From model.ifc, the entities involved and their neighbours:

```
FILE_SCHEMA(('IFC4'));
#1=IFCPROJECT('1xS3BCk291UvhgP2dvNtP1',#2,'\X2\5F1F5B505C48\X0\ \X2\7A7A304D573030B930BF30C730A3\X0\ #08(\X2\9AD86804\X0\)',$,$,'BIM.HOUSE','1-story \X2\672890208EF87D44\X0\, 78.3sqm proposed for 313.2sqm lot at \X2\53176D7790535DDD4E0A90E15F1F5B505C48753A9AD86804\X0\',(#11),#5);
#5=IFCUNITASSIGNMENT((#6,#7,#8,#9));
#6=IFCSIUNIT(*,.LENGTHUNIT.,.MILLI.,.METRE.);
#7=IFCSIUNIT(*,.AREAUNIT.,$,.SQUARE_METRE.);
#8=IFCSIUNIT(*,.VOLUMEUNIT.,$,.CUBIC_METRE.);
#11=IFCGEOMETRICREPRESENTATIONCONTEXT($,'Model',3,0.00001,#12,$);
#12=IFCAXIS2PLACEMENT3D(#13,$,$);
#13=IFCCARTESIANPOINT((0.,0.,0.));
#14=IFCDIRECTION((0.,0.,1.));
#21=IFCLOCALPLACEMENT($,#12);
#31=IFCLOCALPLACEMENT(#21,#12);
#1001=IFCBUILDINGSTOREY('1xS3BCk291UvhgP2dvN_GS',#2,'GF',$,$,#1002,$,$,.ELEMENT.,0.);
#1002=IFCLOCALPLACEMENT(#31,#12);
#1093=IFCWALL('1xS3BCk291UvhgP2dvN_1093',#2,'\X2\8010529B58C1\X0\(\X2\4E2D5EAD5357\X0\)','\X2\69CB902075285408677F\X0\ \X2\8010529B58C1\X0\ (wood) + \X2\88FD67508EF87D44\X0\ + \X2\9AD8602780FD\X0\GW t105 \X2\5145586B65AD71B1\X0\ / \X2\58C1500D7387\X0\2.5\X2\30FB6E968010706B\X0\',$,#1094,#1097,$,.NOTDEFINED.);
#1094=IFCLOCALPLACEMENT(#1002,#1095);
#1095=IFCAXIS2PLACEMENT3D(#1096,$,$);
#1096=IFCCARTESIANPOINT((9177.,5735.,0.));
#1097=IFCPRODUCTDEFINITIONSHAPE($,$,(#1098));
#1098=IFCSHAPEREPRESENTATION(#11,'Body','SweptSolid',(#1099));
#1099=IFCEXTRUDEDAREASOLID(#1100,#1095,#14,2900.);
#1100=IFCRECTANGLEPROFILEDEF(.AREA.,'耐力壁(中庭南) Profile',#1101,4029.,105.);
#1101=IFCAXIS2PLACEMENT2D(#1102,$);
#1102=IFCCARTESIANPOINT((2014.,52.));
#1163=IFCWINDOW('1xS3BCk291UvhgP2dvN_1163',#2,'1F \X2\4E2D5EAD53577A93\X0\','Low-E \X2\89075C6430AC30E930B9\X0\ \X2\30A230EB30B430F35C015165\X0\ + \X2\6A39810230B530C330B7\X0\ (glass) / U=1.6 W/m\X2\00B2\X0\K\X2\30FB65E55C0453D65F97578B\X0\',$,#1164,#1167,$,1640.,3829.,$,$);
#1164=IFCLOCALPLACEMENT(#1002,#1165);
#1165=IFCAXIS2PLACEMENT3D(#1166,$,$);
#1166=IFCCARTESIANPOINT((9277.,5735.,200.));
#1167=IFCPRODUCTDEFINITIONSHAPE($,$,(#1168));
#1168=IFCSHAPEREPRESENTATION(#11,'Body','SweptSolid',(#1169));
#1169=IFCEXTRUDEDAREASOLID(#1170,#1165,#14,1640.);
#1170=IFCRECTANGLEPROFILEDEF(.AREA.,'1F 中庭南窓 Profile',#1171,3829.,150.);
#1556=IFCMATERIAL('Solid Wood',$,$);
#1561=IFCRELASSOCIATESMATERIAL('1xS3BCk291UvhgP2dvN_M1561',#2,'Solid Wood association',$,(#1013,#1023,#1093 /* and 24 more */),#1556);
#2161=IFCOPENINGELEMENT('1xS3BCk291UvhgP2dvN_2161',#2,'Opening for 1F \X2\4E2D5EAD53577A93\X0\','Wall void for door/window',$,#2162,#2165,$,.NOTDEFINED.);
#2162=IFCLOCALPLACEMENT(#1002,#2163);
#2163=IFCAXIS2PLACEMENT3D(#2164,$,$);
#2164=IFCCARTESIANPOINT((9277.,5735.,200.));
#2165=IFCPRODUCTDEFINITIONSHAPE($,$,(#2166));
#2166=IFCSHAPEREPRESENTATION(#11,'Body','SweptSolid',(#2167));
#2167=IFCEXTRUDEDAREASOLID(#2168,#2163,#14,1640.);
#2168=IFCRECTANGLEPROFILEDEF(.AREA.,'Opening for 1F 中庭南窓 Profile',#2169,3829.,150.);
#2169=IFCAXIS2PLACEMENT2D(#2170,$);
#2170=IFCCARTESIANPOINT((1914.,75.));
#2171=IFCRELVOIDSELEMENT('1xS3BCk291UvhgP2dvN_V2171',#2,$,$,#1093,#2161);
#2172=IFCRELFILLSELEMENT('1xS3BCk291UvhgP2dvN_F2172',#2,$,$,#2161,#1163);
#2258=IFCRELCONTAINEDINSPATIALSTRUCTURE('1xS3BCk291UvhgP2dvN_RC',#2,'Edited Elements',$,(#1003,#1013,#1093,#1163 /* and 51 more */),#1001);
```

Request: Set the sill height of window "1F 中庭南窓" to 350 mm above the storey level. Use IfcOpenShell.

```python
import numpy as np
import ifcopenshell
import ifcopenshell.api.geometry
import ifcopenshell.geom
import ifcopenshell.util.element
import ifcopenshell.util.placement
import ifcopenshell.util.shape
import ifcopenshell.util.unit

model = ifcopenshell.open("model.ifc")
unit_scale = ifcopenshell.util.unit.calculate_unit_scale(model)

window = model.by_guid("1xS3BCk291UvhgP2dvN_1163")
opening = window.FillsVoids[0].RelatingOpeningElement
storey = ifcopenshell.util.element.get_container(window, ifc_class="IfcBuildingStorey")
level = ifcopenshell.util.placement.get_local_placement(storey.ObjectPlacement)[2, 3]

# The opening's origin need not be at the sill, so measure its lowest point.
shape = ifcopenshell.geom.create_shape(ifcopenshell.geom.settings(), opening)
bottom = ifcopenshell.util.shape.get_shape_bottom_elevation(shape, shape.geometry) / unit_scale
dz = level + 350.0 - bottom

shift = np.array([0.0, 0.0, dz])
# The window is not placed relative to its opening, so move both.
for product in (opening, window):
    matrix = ifcopenshell.util.placement.get_local_placement(product.ObjectPlacement)
    matrix[:3, 3] += shift
    ifcopenshell.api.geometry.edit_object_placement(model, product=product, matrix=matrix, is_si=False)

print(f"moved by {dz * unit_scale:+.3f} m")

model.write("model_rev.ifc")
```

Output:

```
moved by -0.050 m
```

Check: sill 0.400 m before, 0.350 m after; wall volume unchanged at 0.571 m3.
